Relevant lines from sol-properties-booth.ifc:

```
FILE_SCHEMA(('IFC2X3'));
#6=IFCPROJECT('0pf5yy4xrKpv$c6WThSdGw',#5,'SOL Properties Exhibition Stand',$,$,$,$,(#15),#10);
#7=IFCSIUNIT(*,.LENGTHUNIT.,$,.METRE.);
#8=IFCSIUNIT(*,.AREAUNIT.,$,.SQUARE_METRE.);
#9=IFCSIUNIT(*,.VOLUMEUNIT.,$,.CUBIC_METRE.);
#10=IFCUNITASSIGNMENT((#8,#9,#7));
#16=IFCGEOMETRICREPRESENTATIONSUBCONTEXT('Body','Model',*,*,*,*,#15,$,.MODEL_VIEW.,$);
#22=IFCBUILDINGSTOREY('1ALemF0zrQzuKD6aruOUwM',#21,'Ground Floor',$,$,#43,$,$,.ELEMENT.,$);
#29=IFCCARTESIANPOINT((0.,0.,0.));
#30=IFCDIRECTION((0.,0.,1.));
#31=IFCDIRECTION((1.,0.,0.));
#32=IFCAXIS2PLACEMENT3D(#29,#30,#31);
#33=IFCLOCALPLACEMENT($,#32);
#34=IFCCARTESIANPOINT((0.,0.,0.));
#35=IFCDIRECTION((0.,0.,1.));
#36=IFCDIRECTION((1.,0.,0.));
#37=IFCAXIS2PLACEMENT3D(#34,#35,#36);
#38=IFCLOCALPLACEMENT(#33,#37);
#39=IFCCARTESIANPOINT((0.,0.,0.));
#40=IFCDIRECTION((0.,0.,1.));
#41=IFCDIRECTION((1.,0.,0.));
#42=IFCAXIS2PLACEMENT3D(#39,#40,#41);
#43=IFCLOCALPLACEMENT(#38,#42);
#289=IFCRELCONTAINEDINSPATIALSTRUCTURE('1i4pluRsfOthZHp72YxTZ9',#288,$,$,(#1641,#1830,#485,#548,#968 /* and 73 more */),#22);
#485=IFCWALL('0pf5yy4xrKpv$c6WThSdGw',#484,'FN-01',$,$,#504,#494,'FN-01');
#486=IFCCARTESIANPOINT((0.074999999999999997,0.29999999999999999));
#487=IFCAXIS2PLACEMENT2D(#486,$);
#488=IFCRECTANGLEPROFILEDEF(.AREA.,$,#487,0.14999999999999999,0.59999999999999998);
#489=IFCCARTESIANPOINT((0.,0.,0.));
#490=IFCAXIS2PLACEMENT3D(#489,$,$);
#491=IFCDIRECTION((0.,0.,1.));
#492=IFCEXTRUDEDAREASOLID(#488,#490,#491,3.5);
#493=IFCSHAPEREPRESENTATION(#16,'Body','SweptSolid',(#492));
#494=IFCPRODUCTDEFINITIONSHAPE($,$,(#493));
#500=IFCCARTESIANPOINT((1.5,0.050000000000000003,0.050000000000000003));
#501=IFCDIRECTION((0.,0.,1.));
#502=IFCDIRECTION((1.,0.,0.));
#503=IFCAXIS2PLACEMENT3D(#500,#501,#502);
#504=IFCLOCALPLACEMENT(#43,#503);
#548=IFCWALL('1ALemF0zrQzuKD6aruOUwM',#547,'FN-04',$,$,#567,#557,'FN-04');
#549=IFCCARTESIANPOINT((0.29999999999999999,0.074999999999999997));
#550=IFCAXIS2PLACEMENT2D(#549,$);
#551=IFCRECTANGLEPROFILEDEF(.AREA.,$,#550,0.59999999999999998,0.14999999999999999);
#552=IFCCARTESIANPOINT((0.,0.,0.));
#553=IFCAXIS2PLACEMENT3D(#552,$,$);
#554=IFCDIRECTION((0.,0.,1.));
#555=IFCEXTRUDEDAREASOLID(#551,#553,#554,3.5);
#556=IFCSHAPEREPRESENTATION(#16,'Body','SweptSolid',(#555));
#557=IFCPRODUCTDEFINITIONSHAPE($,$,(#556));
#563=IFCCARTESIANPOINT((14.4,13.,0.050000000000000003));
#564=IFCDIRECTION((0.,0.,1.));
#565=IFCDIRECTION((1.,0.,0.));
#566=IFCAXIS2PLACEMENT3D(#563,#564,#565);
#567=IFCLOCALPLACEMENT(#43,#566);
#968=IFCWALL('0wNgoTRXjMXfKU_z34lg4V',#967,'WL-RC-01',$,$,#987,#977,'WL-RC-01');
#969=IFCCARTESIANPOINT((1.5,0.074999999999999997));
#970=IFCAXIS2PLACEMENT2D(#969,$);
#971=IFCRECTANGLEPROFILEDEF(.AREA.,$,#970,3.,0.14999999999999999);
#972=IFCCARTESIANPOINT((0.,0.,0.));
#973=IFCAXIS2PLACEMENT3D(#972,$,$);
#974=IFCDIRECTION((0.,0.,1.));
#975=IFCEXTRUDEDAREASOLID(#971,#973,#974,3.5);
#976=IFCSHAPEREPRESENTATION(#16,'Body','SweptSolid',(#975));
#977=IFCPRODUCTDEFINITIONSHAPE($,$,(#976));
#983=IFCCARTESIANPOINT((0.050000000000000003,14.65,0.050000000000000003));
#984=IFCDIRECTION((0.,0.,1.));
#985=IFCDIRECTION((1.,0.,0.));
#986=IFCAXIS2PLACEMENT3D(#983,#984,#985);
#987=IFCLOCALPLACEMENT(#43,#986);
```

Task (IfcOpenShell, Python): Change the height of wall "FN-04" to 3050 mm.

```python
import ifcopenshell
import ifcopenshell.geom
import ifcopenshell.util.representation
import ifcopenshell.util.shape

model = ifcopenshell.open("sol-properties-booth.ifc")
settings = ifcopenshell.geom.settings()


def volume(element):
    """Net volume in cubic metres, openings subtracted."""
    shape = ifcopenshell.geom.create_shape(settings, element)
    return ifcopenshell.util.shape.get_volume(shape.geometry)


wall = model.by_id(548)
before = volume(wall)

body = ifcopenshell.util.representation.get_representation(wall, "Model", "Body")
solid = body.Items[0]
old_height = solid.Depth
solid.Depth = 3.05
after = volume(wall)

print(f"height {old_height:g} -> {solid.Depth:g}, volume {before:.3f} -> {after:.3f} m3")

model.write("sol-properties-booth_edited.ifc")
```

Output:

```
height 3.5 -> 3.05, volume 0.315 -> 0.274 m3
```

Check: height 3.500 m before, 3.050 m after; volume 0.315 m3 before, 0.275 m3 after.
